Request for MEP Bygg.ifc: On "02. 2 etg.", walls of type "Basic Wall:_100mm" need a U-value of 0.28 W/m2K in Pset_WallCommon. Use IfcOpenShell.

First a look at what the model holds.

```python
import ifcopenshell
import ifcopenshell.util.element

model = ifcopenshell.open("MEP Bygg.ifc")
print(model.schema)
storey = next(s for s in model.by_type("IfcBuildingStorey") if s.Name == "02. 2 etg.")
walls = [e for e in ifcopenshell.util.element.get_decomposition(storey) if e.is_a("IfcWall")]
seen = {}
for e in walls:
    element_type = ifcopenshell.util.element.get_type(e)
    key = (element_type.Name if element_type != e and element_type else None, ifcopenshell.util.element.get_pset(e, "Pset_WallCommon", "ThermalTransmittance"))
    seen[key] = seen.get(key, 0) + 1
for (name, value), count in sorted(seen.items(), key=str):
    print(count, "x", name, "|", value)
```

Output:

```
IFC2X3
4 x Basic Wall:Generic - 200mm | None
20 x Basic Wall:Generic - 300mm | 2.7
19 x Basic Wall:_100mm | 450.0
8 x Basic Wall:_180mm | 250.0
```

```python
import ifcopenshell
import ifcopenshell.api.pset
import ifcopenshell.util.element

model = ifcopenshell.open("MEP Bygg.ifc")

storey = next(s for s in model.by_type("IfcBuildingStorey") if s.Name == "02. 2 etg.")
walls = [e for e in ifcopenshell.util.element.get_decomposition(storey) if e.is_a("IfcWall")]

count = 0
for e in walls:
    element_type = ifcopenshell.util.element.get_type(e)
    if element_type in (None, e) or element_type.Name != "Basic Wall:_100mm":
        continue
    # add_pset returns the element's existing set when there is one.
    pset = ifcopenshell.api.pset.add_pset(model, product=e, name="Pset_WallCommon")
    ifcopenshell.api.pset.edit_pset(model, pset=pset, properties={"ThermalTransmittance": 0.28})
    count += 1

print(count, "walls updated")

model.write("MEP Bygg-out.ifc")
```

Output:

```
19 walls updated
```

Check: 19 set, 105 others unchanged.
